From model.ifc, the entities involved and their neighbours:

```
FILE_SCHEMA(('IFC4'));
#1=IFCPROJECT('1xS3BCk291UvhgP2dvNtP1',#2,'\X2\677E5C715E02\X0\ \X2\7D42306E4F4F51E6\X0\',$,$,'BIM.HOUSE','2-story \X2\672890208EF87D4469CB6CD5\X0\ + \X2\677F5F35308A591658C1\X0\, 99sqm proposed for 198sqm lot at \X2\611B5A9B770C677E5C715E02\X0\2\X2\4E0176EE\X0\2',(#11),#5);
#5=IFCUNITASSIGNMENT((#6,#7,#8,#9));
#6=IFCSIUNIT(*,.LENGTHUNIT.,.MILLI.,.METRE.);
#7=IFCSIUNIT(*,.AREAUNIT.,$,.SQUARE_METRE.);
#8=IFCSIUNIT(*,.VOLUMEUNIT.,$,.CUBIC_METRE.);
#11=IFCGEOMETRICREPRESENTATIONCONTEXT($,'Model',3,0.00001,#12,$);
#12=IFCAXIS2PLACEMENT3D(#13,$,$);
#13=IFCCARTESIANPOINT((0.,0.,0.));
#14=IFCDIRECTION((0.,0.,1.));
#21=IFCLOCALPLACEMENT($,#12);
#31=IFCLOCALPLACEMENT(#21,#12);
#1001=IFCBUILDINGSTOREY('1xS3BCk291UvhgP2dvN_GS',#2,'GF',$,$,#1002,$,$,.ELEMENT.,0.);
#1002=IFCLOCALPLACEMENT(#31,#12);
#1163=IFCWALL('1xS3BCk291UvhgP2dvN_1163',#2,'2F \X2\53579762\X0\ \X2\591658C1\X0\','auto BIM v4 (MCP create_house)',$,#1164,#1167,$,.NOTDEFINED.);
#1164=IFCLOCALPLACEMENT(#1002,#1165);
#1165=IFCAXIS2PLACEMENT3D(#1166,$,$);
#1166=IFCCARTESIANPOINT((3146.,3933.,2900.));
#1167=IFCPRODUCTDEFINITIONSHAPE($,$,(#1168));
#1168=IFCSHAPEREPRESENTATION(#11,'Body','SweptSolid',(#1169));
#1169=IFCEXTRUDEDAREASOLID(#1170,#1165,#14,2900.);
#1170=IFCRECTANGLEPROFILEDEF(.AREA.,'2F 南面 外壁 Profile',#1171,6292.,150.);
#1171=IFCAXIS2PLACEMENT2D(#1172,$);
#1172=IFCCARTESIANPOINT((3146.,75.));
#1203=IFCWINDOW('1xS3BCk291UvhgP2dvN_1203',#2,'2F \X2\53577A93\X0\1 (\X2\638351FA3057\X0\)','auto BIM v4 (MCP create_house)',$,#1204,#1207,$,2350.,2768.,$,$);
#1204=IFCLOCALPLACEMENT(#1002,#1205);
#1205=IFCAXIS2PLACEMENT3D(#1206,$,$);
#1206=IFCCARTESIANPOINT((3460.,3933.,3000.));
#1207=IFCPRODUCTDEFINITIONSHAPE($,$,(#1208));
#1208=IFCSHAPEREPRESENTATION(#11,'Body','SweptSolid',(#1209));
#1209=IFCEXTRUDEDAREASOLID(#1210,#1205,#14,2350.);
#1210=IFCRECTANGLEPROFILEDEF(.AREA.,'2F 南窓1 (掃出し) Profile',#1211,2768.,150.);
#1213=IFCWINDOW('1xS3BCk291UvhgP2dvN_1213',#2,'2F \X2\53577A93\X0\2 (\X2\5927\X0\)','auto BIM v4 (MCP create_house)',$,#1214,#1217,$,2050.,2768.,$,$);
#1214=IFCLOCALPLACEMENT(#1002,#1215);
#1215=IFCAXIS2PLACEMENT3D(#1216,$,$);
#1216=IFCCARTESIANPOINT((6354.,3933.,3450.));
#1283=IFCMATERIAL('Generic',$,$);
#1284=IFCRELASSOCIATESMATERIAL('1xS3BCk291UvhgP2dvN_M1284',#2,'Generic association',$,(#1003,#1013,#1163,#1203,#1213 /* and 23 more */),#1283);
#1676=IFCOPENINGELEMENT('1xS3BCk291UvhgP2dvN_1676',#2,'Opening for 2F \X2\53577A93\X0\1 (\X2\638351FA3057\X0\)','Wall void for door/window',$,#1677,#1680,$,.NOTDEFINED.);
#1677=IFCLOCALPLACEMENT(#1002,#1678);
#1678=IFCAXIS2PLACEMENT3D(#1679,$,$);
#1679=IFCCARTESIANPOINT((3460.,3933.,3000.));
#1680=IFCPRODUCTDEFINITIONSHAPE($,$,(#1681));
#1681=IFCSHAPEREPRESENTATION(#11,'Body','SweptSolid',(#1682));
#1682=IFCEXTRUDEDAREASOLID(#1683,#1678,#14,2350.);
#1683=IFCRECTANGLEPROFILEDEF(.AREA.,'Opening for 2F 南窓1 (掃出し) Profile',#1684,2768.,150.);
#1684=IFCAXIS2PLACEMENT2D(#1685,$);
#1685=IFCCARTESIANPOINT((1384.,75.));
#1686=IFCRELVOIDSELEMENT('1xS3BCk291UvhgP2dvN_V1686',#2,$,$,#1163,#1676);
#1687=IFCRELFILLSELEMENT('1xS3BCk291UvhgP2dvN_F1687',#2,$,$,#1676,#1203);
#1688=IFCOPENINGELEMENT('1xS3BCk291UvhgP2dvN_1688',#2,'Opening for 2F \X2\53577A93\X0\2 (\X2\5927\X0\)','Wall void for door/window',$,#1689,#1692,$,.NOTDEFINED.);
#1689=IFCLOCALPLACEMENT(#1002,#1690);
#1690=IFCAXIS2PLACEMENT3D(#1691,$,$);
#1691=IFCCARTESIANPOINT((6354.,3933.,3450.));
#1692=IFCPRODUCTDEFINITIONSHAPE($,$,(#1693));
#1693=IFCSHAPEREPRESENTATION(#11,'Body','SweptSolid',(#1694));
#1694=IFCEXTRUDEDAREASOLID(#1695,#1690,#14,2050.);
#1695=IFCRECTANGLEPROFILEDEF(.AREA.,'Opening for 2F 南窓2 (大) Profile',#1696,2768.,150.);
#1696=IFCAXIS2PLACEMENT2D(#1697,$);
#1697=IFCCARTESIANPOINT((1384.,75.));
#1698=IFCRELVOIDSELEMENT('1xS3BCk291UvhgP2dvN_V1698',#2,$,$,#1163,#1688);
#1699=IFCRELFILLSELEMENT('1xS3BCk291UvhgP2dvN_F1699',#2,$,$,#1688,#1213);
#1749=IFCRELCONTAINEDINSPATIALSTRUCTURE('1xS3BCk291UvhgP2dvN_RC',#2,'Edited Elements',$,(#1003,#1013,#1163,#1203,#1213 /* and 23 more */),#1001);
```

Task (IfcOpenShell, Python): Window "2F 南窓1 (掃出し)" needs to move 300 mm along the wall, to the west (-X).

```python
import ifcopenshell
import ifcopenshell.api.geometry
import ifcopenshell.util.placement
import ifcopenshell.util.unit

model = ifcopenshell.open("model.ifc")
unit_scale = ifcopenshell.util.unit.calculate_unit_scale(model)

window = model.by_id(1203)
opening = window.FillsVoids[0].RelatingOpeningElement
wall = opening.VoidsElements[0].RelatingBuildingElement

wall_matrix = ifcopenshell.util.placement.get_local_placement(wall.ObjectPlacement)
shift = wall_matrix[:3, 0] * -0.3 / unit_scale
before = ifcopenshell.util.placement.get_local_placement(window.ObjectPlacement)[:3, 3].copy()

# The window is not placed relative to its opening, so move both.
for product in (opening, window):
    matrix = ifcopenshell.util.placement.get_local_placement(product.ObjectPlacement)
    matrix[:3, 3] += shift
    ifcopenshell.api.geometry.edit_object_placement(model, product=product, matrix=matrix, is_si=False)

after = ifcopenshell.util.placement.get_local_placement(window.ObjectPlacement)[:3, 3]
print("window moved by", (after - before).round(3) + 0.0)

model.write("model_updated.ifc")
```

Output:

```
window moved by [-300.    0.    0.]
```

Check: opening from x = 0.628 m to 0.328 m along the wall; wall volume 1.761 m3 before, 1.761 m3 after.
